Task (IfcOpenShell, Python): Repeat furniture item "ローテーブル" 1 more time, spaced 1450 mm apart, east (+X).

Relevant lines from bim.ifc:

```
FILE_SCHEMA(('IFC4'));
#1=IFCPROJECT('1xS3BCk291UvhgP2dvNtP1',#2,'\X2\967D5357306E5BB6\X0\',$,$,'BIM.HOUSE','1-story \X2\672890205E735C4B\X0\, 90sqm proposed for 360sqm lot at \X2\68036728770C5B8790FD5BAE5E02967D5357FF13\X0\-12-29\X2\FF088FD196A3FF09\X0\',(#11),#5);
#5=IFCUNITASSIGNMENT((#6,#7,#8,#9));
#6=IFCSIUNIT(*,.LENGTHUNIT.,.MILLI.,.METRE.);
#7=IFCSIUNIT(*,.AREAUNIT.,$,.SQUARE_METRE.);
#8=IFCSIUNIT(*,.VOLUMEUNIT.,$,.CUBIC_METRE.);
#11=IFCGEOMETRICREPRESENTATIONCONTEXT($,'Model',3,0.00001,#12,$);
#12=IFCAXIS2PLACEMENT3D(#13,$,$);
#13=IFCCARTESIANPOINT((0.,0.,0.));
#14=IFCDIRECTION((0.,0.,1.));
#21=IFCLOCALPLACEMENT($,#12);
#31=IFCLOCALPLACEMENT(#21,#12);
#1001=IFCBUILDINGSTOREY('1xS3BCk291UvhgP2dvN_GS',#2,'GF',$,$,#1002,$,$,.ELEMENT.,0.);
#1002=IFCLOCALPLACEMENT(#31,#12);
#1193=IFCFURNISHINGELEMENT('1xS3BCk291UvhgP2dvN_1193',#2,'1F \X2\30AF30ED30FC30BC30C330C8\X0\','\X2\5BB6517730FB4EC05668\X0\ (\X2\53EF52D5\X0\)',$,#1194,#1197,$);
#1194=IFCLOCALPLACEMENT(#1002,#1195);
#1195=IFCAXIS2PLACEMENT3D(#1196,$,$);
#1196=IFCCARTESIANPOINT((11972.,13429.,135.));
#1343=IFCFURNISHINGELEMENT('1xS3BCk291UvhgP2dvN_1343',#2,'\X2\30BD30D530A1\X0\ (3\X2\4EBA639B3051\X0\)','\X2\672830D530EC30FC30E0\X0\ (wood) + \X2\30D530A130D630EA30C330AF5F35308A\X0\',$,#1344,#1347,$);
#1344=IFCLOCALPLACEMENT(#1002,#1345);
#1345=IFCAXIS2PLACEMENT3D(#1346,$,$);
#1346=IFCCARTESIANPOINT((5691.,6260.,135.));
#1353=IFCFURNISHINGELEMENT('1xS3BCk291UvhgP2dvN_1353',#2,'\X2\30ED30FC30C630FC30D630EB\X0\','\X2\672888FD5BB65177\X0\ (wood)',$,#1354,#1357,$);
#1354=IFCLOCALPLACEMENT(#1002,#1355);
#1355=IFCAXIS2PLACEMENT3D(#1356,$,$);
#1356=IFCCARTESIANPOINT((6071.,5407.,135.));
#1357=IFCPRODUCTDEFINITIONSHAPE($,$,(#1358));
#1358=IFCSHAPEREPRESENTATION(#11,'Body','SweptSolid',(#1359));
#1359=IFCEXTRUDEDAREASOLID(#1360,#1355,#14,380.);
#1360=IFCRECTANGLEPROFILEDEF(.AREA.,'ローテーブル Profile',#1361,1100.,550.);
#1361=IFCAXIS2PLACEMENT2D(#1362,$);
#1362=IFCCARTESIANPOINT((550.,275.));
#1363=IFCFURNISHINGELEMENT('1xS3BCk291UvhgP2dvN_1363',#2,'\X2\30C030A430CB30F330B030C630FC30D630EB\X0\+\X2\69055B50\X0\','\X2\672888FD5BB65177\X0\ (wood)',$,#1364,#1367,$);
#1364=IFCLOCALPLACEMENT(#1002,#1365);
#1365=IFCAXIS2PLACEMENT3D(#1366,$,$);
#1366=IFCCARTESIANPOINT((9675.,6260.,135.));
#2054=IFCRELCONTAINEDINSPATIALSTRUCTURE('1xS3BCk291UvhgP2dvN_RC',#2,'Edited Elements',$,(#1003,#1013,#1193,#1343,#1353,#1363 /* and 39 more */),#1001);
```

```python
import numpy as np
import ifcopenshell
import ifcopenshell.api.geometry
import ifcopenshell.api.root
import ifcopenshell.util.element
import ifcopenshell.util.placement

model = ifcopenshell.open("bim.ifc")


def reuse_history(source, copy):
    """copy_class also copies each property set's owner history, people and application; keep the originals."""
    for rel in copy.IsDefinedBy:
        if rel.is_a("IfcRelDefinesByProperties") and (history := rel.RelatingPropertyDefinition.OwnerHistory):
            rel.RelatingPropertyDefinition.OwnerHistory = source.OwnerHistory
            ifcopenshell.util.element.remove_deep2(model, history)


source = model.by_id(1353)
base = ifcopenshell.util.placement.get_local_placement(source.ObjectPlacement)
step = np.array([1.0, 0.0, 0.0]) * 1450.0

for i in range(1, 2):
    copy = ifcopenshell.api.root.copy_class(model, product=source)
    copy.Representation = ifcopenshell.util.element.copy_deep(
        model, source.Representation, exclude=["IfcGeometricRepresentationContext", "IfcRepresentationMap"]
    )
    reuse_history(source, copy)
    matrix = base.copy()
    matrix[:3, 3] += i * step
    print("added at", matrix[:3, 3].round(3) + 0.0)
    ifcopenshell.api.geometry.edit_object_placement(model, product=copy, matrix=matrix, is_si=False)

model.write("bim_updated.ifc")
```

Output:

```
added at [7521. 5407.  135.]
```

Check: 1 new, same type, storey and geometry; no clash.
